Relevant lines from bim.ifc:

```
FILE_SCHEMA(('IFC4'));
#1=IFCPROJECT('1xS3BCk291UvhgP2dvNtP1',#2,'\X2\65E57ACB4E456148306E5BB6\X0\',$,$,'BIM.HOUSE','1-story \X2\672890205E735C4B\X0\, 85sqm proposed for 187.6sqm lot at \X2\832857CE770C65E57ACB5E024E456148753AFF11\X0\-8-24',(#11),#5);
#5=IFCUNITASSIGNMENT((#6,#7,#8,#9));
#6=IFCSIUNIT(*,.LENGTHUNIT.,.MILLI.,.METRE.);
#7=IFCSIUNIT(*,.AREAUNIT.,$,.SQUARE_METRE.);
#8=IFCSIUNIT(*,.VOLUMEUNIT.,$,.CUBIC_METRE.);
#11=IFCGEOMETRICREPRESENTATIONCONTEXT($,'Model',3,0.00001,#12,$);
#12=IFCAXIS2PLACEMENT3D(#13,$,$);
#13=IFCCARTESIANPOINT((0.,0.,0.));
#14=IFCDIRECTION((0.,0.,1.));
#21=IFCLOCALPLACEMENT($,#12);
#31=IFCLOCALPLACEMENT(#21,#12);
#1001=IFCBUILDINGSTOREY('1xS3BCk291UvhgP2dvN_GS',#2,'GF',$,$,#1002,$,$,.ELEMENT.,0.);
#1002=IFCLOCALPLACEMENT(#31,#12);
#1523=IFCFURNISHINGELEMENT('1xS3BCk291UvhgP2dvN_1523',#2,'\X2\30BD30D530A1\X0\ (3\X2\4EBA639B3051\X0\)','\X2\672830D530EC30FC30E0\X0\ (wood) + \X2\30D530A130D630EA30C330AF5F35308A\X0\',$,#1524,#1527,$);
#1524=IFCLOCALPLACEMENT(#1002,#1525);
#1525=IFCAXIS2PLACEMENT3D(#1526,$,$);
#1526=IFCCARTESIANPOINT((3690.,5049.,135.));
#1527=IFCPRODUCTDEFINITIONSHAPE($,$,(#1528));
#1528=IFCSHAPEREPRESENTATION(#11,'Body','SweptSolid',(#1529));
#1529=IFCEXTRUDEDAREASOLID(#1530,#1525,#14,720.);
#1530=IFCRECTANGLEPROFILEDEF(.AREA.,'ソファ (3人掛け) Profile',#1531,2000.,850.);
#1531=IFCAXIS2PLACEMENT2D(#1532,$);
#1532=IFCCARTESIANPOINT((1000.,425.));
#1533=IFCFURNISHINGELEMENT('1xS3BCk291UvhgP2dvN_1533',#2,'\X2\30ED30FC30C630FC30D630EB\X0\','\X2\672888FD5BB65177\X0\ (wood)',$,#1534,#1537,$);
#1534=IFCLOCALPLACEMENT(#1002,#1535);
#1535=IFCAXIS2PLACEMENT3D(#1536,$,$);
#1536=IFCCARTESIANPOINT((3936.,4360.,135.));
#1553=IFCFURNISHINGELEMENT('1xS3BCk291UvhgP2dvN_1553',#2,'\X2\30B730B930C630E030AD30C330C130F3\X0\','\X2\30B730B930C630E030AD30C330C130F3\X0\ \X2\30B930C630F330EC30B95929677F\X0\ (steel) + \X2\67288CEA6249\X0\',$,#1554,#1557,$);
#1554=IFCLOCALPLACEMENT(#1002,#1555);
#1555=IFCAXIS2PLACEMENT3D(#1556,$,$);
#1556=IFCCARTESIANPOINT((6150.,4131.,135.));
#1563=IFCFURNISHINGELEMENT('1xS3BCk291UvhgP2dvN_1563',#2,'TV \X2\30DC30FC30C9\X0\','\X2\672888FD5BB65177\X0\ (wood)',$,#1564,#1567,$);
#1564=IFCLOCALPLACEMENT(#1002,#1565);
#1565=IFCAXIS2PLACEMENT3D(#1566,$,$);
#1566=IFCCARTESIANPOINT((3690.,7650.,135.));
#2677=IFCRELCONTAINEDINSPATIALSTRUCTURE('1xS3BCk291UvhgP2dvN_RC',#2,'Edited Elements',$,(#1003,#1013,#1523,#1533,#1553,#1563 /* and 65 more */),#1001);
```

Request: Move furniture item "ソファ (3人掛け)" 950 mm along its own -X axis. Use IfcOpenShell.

```python
import ifcopenshell
import ifcopenshell.api.geometry
import ifcopenshell.util.placement
import ifcopenshell.util.unit

model = ifcopenshell.open("bim.ifc")
unit_scale = ifcopenshell.util.unit.calculate_unit_scale(model)

item = model.by_guid("1xS3BCk291UvhgP2dvN_1523")
matrix = ifcopenshell.util.placement.get_local_placement(item.ObjectPlacement)
matrix[:3, 3] -= matrix[:3, 0] * 0.95 / unit_scale
ifcopenshell.api.geometry.edit_object_placement(model, product=item, matrix=matrix, is_si=False)

print(ifcopenshell.util.placement.get_local_placement(item.ObjectPlacement).round(3) + 0.0)

model.write("bim_edited.ifc")
```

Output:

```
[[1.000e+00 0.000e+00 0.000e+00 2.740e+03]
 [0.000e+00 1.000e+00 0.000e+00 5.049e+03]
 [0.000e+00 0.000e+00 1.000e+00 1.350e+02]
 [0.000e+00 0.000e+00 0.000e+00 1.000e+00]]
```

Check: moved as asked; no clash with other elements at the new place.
